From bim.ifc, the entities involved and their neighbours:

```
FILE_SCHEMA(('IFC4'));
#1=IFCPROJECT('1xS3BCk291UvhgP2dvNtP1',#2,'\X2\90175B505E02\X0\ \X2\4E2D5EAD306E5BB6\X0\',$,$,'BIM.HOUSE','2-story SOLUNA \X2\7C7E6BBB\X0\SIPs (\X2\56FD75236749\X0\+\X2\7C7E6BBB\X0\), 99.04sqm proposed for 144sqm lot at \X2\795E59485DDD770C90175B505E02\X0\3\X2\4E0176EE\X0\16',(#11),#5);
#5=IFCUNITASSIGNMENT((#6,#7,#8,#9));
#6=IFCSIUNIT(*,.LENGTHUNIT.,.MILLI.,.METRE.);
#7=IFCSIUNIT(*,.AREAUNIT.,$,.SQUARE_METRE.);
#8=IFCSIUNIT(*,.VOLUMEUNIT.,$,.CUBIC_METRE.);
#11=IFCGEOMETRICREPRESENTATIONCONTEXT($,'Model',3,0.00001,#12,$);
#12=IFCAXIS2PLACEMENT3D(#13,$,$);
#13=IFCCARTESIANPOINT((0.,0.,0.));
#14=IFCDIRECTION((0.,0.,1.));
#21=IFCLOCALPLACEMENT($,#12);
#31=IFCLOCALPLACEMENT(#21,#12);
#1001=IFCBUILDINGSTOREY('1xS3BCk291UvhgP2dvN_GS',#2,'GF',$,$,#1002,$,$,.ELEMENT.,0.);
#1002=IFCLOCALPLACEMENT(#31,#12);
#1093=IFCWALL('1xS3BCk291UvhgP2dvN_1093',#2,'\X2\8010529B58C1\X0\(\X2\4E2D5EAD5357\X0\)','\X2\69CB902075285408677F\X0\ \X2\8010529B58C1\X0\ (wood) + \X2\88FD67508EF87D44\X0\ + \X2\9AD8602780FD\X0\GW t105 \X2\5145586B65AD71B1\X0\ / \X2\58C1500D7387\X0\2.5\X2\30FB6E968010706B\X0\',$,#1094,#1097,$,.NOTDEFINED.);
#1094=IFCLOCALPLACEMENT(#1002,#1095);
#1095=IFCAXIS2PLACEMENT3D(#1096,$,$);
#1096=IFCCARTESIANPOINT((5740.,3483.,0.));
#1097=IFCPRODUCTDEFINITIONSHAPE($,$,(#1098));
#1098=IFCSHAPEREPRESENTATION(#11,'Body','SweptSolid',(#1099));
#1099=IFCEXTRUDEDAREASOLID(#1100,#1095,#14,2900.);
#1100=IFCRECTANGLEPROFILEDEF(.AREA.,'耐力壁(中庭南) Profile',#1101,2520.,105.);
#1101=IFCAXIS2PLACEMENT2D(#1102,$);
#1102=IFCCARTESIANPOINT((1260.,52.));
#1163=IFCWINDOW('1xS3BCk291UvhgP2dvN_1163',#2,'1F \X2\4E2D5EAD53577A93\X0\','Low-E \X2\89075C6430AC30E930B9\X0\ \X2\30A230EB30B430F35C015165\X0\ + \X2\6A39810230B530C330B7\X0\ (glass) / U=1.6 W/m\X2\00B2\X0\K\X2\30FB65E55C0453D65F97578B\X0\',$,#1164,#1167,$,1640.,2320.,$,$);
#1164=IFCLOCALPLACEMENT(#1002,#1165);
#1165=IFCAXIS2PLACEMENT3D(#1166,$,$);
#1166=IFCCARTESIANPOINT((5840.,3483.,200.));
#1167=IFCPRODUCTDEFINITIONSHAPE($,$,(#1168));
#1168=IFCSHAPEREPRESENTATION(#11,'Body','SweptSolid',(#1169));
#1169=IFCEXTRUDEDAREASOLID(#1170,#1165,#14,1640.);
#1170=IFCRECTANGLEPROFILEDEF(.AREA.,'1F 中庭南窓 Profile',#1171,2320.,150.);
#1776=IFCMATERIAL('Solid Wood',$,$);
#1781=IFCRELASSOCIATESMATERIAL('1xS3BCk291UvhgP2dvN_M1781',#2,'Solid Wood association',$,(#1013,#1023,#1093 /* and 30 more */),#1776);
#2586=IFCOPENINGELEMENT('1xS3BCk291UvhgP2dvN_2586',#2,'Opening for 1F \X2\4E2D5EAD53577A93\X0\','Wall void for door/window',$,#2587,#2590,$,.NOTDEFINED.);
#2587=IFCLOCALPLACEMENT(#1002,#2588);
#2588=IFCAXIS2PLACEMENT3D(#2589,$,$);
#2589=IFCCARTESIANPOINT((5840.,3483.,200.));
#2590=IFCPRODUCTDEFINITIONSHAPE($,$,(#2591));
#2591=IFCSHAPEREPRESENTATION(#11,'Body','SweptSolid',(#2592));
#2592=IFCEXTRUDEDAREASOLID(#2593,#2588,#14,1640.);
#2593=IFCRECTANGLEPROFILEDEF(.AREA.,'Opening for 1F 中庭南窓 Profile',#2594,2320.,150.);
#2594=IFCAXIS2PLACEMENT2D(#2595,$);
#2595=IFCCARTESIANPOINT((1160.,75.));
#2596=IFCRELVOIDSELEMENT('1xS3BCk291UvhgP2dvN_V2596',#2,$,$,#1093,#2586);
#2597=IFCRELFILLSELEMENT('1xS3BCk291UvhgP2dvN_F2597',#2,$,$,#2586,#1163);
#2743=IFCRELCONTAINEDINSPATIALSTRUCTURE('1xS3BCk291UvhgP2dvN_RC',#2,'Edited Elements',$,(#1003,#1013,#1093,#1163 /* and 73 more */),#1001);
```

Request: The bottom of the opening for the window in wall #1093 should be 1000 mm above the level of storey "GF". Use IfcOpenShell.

```python
import numpy as np
import ifcopenshell
import ifcopenshell.api.geometry
import ifcopenshell.geom
import ifcopenshell.util.element
import ifcopenshell.util.placement
import ifcopenshell.util.shape
import ifcopenshell.util.unit

model = ifcopenshell.open("bim.ifc")
unit_scale = ifcopenshell.util.unit.calculate_unit_scale(model)

window = model.by_guid("1xS3BCk291UvhgP2dvN_1163")
opening = window.FillsVoids[0].RelatingOpeningElement
storey = ifcopenshell.util.element.get_container(window, ifc_class="IfcBuildingStorey")
level = ifcopenshell.util.placement.get_local_placement(storey.ObjectPlacement)[2, 3]

# The opening's origin need not be at the sill, so measure its lowest point.
shape = ifcopenshell.geom.create_shape(ifcopenshell.geom.settings(), opening)
bottom = ifcopenshell.util.shape.get_shape_bottom_elevation(shape, shape.geometry) / unit_scale
dz = level + 1 / unit_scale - bottom

shift = np.array([0.0, 0.0, dz])
# The window is not placed relative to its opening, so move both.
for product in (opening, window):
    matrix = ifcopenshell.util.placement.get_local_placement(product.ObjectPlacement)
    matrix[:3, 3] += shift
    ifcopenshell.api.geometry.edit_object_placement(model, product=product, matrix=matrix, is_si=False)

print(f"moved by {dz * unit_scale:+.3f} m")

model.write("bim_rev.ifc")
```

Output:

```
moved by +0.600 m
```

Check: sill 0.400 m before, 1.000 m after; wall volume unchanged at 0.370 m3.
